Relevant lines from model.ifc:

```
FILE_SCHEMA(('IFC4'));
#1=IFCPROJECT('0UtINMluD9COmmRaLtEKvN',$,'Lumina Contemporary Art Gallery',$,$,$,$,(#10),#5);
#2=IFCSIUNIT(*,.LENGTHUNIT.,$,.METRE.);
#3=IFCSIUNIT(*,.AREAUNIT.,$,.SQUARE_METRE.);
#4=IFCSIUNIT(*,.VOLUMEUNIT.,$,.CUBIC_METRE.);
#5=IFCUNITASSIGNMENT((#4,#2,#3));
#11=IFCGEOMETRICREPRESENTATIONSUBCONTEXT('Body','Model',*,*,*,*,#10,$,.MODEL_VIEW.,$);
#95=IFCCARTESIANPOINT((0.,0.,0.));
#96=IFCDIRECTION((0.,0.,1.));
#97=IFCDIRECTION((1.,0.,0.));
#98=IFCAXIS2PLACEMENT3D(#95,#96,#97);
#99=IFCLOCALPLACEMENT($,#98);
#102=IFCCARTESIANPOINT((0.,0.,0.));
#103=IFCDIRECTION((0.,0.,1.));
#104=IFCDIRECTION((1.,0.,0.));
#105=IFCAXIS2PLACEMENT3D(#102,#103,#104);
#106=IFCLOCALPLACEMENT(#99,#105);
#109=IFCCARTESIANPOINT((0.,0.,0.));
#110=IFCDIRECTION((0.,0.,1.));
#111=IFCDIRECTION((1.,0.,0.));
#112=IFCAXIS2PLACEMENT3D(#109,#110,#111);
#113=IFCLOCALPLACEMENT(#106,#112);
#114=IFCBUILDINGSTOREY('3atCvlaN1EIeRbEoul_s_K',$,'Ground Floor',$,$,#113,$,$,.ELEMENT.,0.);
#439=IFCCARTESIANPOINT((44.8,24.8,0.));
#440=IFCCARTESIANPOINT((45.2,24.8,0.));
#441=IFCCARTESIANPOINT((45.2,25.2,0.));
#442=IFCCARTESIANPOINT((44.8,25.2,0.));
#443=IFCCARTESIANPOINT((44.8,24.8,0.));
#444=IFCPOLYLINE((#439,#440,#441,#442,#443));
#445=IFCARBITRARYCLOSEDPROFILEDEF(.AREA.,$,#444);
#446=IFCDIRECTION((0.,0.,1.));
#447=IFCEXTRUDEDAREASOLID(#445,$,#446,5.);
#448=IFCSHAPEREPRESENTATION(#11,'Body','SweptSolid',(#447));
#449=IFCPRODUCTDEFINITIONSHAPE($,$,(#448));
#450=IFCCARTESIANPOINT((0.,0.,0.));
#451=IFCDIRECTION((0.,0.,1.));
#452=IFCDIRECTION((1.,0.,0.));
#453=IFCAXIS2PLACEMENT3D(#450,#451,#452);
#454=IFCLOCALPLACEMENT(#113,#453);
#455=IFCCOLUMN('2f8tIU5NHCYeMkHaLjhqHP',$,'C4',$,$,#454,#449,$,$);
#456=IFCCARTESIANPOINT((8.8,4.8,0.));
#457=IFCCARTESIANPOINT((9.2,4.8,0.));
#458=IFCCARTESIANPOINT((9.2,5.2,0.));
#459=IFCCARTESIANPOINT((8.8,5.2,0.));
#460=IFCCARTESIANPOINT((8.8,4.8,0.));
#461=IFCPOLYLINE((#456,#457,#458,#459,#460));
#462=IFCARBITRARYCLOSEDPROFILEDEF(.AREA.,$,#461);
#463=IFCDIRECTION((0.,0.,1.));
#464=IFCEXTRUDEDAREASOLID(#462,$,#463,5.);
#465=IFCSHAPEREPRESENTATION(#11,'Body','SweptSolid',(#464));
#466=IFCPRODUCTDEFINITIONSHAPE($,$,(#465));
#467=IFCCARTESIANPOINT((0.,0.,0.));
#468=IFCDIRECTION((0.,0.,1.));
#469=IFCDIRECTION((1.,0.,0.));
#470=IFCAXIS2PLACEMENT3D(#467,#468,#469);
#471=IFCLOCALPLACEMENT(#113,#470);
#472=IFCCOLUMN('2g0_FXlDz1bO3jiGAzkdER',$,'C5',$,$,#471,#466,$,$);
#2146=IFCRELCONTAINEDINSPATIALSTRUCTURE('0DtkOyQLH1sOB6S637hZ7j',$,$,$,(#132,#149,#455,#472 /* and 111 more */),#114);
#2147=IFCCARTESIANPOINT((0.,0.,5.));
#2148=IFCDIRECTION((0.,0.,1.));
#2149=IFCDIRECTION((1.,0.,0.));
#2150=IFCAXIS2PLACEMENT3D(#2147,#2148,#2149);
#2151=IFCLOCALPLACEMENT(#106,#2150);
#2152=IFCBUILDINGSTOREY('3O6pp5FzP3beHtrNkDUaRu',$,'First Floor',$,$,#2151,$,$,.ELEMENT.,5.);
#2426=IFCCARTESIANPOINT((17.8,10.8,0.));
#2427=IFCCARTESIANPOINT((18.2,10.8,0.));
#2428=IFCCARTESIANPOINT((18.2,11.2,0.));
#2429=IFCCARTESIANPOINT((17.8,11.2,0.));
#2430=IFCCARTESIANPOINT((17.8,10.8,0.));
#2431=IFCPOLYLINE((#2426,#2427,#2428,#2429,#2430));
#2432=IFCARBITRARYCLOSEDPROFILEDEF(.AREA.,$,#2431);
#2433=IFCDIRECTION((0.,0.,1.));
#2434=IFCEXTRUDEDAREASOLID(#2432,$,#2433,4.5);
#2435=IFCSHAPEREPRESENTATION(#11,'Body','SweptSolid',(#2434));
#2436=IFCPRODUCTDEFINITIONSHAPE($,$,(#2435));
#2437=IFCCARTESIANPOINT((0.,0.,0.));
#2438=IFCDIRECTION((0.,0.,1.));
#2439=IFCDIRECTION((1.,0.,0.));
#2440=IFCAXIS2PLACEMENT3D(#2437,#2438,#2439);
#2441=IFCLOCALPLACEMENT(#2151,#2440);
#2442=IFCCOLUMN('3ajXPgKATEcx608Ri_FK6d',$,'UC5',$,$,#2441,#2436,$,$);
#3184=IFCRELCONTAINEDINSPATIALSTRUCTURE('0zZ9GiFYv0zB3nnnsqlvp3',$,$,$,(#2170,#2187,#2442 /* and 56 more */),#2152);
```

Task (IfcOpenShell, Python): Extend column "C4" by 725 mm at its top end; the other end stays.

```python
import ifcopenshell
import ifcopenshell.util.representation

model = ifcopenshell.open("model.ifc")

member = model.by_guid("2f8tIU5NHCYeMkHaLjhqHP")
change = 0.725

# The extrusion runs towards the end named, so only its depth changes.
body = ifcopenshell.util.representation.get_representation(member, "Model", "Body")
solid = body.Items[0]
old_length = solid.Depth
solid.Depth += change

print(f"length {old_length:g} -> {solid.Depth:g}")

model.write("model-out.ifc")
```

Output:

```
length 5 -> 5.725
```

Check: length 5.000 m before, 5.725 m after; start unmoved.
